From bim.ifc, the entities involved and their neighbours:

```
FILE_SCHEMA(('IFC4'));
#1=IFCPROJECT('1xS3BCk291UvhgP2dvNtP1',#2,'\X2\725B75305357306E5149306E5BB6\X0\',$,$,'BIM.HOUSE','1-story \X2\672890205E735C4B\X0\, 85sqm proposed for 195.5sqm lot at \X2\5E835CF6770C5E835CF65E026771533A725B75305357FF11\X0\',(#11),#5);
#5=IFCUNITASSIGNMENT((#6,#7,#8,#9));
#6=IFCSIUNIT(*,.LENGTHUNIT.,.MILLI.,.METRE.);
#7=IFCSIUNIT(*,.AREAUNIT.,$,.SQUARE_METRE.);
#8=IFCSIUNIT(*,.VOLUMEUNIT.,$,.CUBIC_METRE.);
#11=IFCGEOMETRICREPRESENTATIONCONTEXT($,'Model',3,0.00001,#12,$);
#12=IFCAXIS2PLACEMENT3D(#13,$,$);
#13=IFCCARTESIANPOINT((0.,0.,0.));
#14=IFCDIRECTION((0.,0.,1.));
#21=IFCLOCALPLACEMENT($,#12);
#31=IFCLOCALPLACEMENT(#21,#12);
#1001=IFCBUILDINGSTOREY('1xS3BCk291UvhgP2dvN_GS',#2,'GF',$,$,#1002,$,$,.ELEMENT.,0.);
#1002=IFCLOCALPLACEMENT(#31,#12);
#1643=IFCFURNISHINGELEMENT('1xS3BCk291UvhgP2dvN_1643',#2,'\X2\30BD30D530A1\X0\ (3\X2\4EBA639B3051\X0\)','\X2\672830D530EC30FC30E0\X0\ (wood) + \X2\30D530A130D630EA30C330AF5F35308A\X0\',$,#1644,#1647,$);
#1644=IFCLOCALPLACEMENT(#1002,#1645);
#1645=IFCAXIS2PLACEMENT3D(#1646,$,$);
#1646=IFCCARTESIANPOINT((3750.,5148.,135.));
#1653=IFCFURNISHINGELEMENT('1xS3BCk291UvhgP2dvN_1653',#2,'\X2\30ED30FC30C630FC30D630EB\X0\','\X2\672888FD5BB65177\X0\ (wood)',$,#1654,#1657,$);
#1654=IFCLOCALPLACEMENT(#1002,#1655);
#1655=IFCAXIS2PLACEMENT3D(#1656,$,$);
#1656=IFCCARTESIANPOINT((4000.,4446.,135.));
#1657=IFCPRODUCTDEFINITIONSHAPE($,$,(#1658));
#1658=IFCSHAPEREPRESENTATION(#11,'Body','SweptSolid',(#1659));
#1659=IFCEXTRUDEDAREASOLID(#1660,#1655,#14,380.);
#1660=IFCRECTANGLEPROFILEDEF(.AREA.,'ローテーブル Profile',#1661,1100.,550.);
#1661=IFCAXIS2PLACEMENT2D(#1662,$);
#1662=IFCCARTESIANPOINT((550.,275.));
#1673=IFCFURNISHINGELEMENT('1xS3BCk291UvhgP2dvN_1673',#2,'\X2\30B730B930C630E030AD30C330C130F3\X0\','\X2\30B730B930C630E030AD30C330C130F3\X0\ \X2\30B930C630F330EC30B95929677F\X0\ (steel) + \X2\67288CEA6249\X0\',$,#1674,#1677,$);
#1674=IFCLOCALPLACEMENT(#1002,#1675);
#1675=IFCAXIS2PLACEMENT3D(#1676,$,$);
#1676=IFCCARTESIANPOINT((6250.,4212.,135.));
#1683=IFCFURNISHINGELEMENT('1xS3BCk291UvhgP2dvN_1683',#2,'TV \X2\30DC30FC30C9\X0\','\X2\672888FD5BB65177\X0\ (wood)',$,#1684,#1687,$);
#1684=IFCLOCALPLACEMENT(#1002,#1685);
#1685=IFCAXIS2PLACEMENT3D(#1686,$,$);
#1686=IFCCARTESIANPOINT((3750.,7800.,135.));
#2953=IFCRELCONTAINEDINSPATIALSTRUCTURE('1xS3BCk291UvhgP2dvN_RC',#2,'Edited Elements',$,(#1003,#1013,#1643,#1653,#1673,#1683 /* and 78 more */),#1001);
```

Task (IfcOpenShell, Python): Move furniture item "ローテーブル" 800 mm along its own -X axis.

```python
import ifcopenshell
import ifcopenshell.api.geometry
import ifcopenshell.util.placement
import ifcopenshell.util.unit

model = ifcopenshell.open("bim.ifc")
unit_scale = ifcopenshell.util.unit.calculate_unit_scale(model)

item = model.by_id(1653)
matrix = ifcopenshell.util.placement.get_local_placement(item.ObjectPlacement)
matrix[:3, 3] -= matrix[:3, 0] * 0.8 / unit_scale
ifcopenshell.api.geometry.edit_object_placement(model, product=item, matrix=matrix, is_si=False)

print(ifcopenshell.util.placement.get_local_placement(item.ObjectPlacement).round(3) + 0.0)

model.write("bim-out.ifc")
```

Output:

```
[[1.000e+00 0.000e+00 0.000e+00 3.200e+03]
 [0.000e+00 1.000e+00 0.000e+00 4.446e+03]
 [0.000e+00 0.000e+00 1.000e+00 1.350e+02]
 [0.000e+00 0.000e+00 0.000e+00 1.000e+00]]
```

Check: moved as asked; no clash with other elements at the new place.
